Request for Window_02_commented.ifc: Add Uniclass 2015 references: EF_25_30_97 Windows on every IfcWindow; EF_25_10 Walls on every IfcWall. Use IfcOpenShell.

First a look at what the model holds.

```python
import ifcopenshell

model = ifcopenshell.open("Window_02_commented.ifc")
print(model.schema)
print("classifications:", [c.Name for c in model.by_type("IfcClassification")])
for ifc_class in ("IfcDoor", "IfcRoof", "IfcStair", "IfcWall", "IfcWindow"):
    print(ifc_class, len(model.by_type(ifc_class)))
```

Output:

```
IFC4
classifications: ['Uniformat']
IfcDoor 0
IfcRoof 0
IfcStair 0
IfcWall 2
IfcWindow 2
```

```python
import ifcopenshell
import ifcopenshell.api.classification

model = ifcopenshell.open("Window_02_commented.ifc")

system = ifcopenshell.api.classification.add_classification(model, classification="Uniclass 2015")

codes = {
    "IfcWindow": ("EF_25_30_97", "Windows"),
    "IfcWall": ("EF_25_10", "Walls"),
}
for ifc_class, (code, name) in codes.items():
    products = model.by_type(ifc_class)
    ifcopenshell.api.classification.add_reference(
        model, products=products, classification=system, identification=code, name=name
    )
    print(code, len(products))

model.write("Window_02_commented_updated.ifc")
```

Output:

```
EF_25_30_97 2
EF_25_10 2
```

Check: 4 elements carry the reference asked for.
